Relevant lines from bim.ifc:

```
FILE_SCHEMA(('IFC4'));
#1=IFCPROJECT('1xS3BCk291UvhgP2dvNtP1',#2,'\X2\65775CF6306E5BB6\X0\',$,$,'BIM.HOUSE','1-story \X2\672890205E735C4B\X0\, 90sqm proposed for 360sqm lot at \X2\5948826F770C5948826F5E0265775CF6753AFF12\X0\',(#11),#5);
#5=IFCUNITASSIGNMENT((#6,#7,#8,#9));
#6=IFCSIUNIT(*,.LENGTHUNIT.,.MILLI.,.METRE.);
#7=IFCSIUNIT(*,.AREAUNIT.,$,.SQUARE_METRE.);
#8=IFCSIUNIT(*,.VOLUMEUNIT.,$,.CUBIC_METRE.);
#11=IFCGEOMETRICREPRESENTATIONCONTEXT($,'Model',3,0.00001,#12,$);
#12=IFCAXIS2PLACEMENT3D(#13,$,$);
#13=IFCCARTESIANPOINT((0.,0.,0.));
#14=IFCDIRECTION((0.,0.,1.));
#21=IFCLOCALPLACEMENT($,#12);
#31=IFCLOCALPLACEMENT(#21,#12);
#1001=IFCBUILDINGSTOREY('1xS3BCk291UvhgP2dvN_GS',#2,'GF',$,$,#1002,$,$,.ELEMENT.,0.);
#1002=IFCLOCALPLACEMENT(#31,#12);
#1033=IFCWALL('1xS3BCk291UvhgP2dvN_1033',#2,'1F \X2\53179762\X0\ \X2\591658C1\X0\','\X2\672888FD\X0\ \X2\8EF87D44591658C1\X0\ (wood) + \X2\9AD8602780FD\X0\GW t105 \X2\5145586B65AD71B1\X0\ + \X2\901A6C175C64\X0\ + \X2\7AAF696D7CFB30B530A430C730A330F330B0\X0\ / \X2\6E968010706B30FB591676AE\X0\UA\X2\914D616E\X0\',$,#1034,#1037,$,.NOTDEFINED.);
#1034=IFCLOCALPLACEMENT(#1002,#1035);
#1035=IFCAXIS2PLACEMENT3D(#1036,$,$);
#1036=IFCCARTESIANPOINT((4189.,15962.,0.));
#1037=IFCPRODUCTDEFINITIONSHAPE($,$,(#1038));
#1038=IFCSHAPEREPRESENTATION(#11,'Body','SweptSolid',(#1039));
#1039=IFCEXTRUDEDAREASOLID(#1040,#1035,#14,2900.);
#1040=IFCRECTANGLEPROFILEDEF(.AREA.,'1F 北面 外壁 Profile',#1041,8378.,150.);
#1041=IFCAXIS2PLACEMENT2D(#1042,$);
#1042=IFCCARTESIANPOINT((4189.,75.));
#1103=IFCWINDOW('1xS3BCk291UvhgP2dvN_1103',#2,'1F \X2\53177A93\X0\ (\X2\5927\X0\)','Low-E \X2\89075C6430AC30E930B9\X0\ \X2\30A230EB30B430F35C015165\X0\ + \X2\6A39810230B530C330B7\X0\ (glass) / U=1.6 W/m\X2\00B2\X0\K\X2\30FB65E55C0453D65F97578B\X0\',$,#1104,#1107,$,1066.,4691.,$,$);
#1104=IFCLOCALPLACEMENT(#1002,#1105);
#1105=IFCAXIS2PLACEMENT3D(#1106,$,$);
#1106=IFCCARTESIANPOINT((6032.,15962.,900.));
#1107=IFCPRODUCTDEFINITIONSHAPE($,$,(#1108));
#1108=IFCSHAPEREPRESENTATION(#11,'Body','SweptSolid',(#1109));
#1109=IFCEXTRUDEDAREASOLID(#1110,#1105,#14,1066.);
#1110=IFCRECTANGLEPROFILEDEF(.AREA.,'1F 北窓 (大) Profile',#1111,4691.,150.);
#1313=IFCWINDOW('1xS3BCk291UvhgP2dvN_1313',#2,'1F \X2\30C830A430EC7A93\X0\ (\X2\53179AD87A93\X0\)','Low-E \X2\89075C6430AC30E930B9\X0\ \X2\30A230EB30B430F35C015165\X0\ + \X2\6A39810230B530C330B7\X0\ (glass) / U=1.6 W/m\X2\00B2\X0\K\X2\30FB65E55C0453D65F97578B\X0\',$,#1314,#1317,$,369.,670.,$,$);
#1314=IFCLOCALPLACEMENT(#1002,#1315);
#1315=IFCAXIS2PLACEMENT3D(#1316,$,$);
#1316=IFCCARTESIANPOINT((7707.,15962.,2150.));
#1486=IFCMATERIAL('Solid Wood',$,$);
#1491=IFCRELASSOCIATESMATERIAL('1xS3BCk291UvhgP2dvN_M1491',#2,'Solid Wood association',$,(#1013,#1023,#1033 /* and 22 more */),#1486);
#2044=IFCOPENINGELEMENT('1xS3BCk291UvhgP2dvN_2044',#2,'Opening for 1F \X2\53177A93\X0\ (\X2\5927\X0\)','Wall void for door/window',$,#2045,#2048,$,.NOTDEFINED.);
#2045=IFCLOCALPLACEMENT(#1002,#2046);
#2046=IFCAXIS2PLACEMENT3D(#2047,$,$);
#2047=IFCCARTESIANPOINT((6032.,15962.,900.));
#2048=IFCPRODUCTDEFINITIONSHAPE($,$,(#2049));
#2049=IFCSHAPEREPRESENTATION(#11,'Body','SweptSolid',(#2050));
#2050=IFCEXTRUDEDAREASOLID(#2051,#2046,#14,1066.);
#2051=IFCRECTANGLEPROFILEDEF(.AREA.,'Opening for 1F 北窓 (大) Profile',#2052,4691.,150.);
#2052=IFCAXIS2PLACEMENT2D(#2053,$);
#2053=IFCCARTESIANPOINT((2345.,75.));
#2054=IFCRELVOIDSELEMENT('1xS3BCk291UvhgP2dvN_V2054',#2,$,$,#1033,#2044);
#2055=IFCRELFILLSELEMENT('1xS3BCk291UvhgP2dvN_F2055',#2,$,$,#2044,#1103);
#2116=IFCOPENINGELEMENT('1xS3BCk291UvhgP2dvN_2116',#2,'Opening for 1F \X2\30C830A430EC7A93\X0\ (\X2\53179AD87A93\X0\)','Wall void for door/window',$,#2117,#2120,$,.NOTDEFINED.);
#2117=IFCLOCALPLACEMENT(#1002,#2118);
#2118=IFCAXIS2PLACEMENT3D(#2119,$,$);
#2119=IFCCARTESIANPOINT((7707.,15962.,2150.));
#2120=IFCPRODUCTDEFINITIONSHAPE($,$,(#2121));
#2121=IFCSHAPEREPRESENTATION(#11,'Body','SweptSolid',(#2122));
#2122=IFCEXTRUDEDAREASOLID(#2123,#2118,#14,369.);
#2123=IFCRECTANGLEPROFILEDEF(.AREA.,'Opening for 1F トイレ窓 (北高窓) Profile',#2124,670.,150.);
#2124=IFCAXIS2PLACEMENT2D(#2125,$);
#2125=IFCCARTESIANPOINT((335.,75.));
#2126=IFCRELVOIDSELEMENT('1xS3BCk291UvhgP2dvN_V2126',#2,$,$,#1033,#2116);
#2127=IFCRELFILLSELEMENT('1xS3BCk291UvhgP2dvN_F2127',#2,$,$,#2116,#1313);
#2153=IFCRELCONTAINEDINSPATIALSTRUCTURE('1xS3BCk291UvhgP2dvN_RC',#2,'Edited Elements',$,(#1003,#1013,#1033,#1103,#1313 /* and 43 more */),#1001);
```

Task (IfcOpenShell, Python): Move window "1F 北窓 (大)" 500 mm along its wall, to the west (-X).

```python
import ifcopenshell
import ifcopenshell.api.geometry
import ifcopenshell.util.placement
import ifcopenshell.util.unit

model = ifcopenshell.open("bim.ifc")
unit_scale = ifcopenshell.util.unit.calculate_unit_scale(model)

window = model.by_id(1103)
opening = window.FillsVoids[0].RelatingOpeningElement
wall = opening.VoidsElements[0].RelatingBuildingElement

wall_matrix = ifcopenshell.util.placement.get_local_placement(wall.ObjectPlacement)
shift = wall_matrix[:3, 0] * -0.5 / unit_scale
before = ifcopenshell.util.placement.get_local_placement(window.ObjectPlacement)[:3, 3].copy()

# The window is not placed relative to its opening, so move both.
for product in (opening, window):
    matrix = ifcopenshell.util.placement.get_local_placement(product.ObjectPlacement)
    matrix[:3, 3] += shift
    ifcopenshell.api.geometry.edit_object_placement(model, product=product, matrix=matrix, is_si=False)

after = ifcopenshell.util.placement.get_local_placement(window.ObjectPlacement)[:3, 3]
print("window moved by", (after - before).round(3) + 0.0)

model.write("bim-out.ifc")
```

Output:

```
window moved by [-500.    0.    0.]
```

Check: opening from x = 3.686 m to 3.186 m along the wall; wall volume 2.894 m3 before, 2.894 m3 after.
